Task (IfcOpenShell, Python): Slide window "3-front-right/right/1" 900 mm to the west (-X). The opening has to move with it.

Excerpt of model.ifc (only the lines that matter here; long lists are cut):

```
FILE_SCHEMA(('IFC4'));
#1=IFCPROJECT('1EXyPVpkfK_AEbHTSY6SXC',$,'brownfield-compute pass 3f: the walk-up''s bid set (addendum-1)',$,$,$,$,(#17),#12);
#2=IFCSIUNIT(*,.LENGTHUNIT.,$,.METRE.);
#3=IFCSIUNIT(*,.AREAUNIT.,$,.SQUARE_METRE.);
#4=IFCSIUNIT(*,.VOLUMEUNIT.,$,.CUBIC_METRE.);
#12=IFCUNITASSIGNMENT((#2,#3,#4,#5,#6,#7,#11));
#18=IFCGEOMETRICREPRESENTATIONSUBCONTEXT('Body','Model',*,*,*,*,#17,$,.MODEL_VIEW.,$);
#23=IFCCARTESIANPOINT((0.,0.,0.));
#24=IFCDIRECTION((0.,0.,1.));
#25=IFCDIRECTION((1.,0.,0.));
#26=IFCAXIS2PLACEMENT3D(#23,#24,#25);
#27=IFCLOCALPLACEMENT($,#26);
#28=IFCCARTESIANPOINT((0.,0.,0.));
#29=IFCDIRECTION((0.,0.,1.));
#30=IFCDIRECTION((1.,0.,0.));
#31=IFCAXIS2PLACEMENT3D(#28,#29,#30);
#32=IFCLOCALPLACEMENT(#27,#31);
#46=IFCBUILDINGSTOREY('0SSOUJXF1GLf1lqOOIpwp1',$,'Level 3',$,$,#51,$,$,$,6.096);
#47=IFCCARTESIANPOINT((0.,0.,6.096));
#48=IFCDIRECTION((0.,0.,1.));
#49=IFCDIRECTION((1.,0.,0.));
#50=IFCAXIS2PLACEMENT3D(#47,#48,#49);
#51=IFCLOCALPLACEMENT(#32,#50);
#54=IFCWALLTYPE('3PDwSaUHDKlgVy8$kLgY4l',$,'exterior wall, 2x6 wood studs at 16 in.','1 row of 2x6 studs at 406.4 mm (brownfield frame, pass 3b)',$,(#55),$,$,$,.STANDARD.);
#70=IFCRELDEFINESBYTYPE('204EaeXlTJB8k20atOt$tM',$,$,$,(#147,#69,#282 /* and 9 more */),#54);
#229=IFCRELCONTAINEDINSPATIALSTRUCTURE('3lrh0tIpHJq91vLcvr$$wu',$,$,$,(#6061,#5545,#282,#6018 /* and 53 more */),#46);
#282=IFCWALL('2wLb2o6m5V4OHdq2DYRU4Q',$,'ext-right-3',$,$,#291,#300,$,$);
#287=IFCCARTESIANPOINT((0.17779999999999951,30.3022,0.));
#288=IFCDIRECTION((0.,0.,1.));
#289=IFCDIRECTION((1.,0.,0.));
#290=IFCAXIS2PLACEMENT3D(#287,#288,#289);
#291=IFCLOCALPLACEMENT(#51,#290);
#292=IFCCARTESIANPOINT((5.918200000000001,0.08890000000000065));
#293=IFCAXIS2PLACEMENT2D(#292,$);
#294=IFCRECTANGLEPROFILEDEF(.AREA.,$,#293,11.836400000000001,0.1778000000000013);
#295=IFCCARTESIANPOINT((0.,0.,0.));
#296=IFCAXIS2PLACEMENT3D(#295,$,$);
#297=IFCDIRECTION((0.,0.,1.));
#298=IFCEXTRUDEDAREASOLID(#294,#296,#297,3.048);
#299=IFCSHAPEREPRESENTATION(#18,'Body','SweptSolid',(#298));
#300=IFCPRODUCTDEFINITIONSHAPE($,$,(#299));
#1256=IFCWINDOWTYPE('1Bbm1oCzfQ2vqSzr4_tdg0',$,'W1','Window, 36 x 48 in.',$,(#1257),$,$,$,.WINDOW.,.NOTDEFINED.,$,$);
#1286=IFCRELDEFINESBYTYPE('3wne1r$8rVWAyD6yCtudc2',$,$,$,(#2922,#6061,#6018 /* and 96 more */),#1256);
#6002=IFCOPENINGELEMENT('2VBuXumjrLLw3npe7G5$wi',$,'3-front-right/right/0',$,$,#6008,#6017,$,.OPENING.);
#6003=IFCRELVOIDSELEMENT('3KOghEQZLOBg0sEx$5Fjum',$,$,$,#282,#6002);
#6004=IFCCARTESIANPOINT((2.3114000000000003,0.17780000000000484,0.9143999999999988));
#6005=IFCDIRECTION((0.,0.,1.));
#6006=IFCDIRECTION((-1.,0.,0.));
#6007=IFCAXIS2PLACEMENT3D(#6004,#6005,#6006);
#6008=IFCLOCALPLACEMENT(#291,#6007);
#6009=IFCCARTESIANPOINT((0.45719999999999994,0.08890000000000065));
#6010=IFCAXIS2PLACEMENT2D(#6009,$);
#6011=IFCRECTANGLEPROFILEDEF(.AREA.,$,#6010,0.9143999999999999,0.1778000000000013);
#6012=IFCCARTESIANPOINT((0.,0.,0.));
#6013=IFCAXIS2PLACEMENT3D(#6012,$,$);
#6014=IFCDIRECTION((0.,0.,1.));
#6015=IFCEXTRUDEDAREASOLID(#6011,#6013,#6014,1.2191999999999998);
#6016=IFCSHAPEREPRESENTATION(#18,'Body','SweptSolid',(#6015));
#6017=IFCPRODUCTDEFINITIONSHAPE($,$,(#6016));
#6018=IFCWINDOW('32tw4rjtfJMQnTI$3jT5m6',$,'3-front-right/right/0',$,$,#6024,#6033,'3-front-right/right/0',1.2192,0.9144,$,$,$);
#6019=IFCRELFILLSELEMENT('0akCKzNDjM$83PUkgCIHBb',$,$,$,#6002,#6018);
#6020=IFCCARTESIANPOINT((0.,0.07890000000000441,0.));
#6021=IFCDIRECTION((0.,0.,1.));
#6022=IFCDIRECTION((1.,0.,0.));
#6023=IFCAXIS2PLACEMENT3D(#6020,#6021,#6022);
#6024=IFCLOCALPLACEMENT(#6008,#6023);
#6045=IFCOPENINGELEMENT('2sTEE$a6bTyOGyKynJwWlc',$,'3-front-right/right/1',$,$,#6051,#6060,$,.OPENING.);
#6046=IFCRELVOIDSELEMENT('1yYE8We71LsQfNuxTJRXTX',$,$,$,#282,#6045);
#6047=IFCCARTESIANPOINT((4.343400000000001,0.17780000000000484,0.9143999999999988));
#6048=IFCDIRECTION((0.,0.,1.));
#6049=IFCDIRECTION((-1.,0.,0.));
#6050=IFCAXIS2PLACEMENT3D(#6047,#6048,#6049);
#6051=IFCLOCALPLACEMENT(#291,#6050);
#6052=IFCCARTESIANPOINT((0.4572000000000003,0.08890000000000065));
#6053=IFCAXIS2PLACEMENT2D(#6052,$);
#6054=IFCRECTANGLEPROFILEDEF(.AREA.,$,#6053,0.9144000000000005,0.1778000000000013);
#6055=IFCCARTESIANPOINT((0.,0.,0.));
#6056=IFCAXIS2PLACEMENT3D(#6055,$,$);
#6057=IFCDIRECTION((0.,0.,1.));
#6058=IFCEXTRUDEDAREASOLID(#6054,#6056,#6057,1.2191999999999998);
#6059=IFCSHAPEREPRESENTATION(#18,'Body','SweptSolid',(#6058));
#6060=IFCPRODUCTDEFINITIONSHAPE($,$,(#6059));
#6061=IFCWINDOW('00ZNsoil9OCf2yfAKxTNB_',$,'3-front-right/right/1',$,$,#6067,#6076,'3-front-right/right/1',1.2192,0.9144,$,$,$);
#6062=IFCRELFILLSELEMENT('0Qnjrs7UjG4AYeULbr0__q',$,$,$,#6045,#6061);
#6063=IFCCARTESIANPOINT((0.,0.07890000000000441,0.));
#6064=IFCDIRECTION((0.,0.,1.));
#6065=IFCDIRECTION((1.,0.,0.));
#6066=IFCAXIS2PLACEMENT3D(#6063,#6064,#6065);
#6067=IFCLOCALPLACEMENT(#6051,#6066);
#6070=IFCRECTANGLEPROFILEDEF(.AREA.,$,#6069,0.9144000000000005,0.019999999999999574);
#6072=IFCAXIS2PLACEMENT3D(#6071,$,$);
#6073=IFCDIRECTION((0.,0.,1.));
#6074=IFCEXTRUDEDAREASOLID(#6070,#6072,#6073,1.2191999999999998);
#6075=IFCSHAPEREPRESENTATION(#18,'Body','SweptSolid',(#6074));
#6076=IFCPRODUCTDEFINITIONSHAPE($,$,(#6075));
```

```python
import ifcopenshell
import ifcopenshell.api.geometry
import ifcopenshell.util.placement
import ifcopenshell.util.unit

model = ifcopenshell.open("model.ifc")
unit_scale = ifcopenshell.util.unit.calculate_unit_scale(model)

window = model.by_guid("00ZNsoil9OCf2yfAKxTNB_")
opening = window.FillsVoids[0].RelatingOpeningElement
wall = opening.VoidsElements[0].RelatingBuildingElement

wall_matrix = ifcopenshell.util.placement.get_local_placement(wall.ObjectPlacement)
shift = wall_matrix[:3, 0] * -0.9 / unit_scale
before = ifcopenshell.util.placement.get_local_placement(window.ObjectPlacement)[:3, 3].copy()

# The window is placed relative to its opening, so it follows when the opening moves.
matrix = ifcopenshell.util.placement.get_local_placement(opening.ObjectPlacement)
matrix[:3, 3] += shift
ifcopenshell.api.geometry.edit_object_placement(
    model, product=opening, matrix=matrix, is_si=False, should_transform_children=True
)

after = ifcopenshell.util.placement.get_local_placement(window.ObjectPlacement)[:3, 3]
print("window moved by", (after - before).round(3) + 0.0)

model.write("model_v2.ifc")
```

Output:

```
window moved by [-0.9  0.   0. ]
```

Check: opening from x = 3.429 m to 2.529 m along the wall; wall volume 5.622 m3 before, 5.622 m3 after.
